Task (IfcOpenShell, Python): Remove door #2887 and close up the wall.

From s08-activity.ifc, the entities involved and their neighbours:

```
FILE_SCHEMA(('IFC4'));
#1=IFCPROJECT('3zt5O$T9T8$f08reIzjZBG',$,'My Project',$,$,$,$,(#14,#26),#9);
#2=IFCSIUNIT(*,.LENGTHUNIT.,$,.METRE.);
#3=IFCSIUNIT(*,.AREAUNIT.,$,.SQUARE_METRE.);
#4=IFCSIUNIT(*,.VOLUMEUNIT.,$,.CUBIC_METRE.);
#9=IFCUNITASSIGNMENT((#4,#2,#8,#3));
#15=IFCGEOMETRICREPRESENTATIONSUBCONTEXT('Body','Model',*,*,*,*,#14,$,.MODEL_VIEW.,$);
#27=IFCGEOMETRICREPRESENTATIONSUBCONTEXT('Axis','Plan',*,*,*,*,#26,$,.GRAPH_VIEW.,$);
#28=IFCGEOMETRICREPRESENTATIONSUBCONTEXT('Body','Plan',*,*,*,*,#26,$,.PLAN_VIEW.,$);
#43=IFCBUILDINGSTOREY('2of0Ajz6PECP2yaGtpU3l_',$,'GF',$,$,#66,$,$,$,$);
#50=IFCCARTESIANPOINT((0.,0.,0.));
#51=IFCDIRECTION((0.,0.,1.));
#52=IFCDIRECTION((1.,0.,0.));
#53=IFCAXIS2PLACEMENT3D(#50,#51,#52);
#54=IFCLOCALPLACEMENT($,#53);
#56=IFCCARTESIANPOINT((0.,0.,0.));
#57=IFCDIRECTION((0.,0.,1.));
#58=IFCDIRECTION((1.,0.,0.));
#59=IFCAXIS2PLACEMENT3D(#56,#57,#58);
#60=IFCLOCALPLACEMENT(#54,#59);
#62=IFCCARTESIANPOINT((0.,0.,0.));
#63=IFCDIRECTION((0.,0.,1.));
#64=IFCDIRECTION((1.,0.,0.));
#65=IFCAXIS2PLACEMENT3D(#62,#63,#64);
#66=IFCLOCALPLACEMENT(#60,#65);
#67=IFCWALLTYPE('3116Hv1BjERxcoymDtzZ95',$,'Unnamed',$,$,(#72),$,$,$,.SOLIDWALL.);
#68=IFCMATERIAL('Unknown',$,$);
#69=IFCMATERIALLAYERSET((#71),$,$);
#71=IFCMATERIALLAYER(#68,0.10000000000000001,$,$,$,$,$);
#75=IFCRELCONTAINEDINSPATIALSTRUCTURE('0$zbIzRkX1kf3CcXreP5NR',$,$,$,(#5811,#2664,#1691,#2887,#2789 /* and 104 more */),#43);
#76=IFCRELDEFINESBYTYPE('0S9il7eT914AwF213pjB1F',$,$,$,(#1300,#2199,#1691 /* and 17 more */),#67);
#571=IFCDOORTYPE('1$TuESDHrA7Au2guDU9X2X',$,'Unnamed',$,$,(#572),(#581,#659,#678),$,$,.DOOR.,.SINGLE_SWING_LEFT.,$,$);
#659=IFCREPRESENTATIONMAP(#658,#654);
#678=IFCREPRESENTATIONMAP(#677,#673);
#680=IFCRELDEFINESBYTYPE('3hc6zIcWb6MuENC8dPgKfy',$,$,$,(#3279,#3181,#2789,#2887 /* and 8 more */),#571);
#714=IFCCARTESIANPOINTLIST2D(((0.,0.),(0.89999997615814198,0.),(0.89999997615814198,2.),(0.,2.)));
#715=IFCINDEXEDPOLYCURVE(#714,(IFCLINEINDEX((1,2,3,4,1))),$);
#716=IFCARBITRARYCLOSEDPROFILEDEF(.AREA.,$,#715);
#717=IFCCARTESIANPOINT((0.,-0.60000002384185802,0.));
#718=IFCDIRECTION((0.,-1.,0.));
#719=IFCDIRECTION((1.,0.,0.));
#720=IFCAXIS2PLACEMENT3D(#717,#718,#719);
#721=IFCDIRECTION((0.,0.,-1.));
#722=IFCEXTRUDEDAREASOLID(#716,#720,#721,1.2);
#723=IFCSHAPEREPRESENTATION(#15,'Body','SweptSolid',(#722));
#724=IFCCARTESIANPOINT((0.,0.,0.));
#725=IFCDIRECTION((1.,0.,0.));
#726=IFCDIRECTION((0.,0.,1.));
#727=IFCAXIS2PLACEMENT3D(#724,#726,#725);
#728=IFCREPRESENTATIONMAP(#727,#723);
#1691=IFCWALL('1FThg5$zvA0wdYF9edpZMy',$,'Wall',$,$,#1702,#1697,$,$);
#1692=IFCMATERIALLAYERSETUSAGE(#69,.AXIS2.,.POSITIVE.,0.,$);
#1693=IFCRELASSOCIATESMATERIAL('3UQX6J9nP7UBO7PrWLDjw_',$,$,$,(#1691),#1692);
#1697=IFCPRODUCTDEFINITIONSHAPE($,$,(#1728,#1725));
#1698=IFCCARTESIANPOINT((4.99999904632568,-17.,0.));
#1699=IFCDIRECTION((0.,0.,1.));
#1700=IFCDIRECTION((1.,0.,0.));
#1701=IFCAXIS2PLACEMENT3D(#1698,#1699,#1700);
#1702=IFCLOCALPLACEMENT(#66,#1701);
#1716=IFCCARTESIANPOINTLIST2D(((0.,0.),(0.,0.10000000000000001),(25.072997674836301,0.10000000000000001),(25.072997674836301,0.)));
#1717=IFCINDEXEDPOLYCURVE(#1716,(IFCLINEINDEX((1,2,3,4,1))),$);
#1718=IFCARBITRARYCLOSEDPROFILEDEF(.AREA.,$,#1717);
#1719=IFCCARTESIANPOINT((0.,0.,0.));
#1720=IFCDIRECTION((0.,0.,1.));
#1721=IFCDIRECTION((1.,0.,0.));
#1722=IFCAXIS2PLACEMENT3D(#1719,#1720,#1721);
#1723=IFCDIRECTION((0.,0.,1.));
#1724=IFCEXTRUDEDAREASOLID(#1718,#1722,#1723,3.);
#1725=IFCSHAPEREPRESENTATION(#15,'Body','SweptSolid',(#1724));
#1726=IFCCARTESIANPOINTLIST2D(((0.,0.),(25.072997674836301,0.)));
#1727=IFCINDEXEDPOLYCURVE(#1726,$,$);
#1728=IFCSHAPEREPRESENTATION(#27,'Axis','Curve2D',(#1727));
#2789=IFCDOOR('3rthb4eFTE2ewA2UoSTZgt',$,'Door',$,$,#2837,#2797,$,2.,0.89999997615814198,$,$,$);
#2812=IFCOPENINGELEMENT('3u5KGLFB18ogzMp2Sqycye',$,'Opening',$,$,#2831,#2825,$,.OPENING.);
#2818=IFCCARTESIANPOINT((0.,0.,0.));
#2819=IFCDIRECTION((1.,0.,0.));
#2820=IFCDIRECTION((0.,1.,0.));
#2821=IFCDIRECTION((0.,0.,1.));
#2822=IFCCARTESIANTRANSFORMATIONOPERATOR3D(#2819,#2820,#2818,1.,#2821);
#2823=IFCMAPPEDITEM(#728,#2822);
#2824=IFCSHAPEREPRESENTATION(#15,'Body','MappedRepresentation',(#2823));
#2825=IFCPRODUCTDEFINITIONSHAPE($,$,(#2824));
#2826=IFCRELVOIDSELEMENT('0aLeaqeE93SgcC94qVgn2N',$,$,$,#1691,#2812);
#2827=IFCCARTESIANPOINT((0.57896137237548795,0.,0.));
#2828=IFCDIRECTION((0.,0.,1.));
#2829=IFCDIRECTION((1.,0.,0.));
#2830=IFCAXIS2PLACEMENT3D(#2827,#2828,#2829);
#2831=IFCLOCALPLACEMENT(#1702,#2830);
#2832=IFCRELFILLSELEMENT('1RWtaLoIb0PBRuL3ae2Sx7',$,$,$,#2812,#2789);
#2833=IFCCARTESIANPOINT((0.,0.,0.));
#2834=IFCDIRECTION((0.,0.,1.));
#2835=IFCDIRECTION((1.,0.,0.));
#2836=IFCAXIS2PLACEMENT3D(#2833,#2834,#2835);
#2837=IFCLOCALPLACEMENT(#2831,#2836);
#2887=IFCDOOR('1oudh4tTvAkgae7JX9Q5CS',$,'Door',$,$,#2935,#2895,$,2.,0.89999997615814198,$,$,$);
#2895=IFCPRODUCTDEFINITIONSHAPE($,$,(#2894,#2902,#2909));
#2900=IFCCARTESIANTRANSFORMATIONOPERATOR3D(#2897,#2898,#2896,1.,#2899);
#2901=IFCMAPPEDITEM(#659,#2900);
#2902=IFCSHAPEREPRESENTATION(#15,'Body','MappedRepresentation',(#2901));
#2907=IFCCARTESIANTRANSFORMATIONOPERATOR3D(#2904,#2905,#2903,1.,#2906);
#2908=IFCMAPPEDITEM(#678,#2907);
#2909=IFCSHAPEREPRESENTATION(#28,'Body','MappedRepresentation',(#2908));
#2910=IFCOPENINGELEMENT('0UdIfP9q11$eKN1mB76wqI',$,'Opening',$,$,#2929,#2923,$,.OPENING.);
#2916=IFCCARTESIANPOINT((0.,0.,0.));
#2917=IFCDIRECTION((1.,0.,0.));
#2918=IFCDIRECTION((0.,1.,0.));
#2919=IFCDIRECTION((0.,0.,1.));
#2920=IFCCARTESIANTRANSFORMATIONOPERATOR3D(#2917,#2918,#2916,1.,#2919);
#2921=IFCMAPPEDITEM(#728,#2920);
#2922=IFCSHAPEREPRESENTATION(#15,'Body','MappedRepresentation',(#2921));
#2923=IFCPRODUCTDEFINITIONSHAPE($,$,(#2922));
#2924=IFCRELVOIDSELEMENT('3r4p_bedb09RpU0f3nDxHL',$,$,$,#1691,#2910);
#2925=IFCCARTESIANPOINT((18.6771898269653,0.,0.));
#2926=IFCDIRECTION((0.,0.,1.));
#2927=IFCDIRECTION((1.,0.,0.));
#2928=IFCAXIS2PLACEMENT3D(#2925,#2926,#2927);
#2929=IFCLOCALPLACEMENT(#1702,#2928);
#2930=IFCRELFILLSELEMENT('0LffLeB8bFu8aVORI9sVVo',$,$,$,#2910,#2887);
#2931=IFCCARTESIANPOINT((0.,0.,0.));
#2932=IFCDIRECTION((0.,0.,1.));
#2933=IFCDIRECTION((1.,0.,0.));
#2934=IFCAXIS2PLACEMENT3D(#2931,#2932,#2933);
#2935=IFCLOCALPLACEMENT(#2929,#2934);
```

```python
import ifcopenshell
import ifcopenshell.api.feature
import ifcopenshell.api.root
import ifcopenshell.geom
import ifcopenshell.util.shape

model = ifcopenshell.open("s08-activity.ifc")
settings = ifcopenshell.geom.settings()


def volume(element):
    """Net volume in cubic metres, openings subtracted."""
    shape = ifcopenshell.geom.create_shape(settings, element)
    return ifcopenshell.util.shape.get_volume(shape.geometry)


door = model.by_id(2887)
opening = door.FillsVoids[0].RelatingOpeningElement
wall = opening.VoidsElements[0].RelatingBuildingElement
before = volume(wall)

ifcopenshell.api.root.remove_product(model, product=door)
ifcopenshell.api.feature.remove_feature(model, feature=opening)

after = volume(wall)

print(f"wall volume {before:.3f} -> {after:.3f} m3")

model.write("s08-activity_edited.ifc")
```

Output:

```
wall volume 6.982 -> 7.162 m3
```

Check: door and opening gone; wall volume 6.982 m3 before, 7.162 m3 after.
